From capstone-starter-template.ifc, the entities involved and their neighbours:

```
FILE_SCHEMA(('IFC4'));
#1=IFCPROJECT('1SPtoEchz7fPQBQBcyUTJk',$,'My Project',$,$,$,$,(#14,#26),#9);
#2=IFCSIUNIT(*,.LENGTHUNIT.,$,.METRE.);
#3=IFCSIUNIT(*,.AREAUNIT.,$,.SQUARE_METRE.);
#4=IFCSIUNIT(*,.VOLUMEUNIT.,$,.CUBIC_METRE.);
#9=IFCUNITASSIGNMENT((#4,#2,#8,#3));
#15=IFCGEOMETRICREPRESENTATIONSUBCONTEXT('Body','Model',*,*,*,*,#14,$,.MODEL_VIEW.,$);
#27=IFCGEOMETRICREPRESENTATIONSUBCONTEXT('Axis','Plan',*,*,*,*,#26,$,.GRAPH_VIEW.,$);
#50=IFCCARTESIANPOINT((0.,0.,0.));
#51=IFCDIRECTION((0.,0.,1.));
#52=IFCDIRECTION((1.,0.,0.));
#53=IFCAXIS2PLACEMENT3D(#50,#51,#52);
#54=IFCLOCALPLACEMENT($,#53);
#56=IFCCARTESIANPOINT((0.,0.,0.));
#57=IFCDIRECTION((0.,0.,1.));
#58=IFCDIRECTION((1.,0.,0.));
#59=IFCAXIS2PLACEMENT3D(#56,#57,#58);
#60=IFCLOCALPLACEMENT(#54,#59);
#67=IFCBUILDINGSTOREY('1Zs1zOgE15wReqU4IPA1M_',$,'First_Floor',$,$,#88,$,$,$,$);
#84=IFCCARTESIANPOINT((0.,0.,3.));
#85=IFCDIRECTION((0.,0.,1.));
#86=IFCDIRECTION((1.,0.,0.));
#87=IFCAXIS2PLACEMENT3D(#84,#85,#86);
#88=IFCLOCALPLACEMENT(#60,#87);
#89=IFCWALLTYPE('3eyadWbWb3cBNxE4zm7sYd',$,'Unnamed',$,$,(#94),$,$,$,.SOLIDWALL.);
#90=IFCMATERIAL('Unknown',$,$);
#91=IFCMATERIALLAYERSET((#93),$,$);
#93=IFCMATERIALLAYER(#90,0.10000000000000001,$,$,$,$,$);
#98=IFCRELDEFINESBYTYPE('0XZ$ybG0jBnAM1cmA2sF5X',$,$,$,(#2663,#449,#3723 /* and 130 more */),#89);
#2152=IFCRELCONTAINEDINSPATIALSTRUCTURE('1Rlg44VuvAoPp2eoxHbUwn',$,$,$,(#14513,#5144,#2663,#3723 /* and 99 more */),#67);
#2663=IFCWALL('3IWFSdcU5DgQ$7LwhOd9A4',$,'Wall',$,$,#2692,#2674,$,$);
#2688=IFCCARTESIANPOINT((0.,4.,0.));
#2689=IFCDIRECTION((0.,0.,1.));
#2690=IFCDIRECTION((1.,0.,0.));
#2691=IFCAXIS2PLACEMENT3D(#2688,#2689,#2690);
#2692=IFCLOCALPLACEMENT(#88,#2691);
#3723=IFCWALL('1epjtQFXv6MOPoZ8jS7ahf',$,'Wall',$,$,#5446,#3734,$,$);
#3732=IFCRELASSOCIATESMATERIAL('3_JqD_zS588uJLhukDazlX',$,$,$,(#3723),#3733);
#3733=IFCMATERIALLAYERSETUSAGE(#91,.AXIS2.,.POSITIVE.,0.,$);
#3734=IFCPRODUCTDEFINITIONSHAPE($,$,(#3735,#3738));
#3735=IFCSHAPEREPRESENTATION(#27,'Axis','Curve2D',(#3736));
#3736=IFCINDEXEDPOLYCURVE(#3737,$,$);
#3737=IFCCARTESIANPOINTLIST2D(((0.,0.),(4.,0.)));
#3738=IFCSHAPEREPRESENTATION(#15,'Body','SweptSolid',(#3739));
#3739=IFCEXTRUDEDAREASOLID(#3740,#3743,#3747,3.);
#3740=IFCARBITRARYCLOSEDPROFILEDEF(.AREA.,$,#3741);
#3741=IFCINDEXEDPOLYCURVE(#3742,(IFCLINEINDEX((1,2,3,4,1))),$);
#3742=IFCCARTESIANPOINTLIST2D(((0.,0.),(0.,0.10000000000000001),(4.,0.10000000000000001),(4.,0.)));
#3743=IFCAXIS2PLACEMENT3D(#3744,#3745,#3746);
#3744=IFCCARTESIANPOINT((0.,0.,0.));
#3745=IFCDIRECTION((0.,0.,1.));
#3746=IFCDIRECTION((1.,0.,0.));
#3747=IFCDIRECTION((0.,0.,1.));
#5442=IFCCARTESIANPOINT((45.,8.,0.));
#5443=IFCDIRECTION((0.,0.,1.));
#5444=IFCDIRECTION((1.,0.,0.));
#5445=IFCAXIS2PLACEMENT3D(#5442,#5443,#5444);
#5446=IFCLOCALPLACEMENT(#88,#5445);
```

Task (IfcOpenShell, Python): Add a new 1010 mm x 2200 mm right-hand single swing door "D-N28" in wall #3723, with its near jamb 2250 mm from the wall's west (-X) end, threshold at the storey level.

```python
import numpy as np
import ifcopenshell
import ifcopenshell.api.feature
import ifcopenshell.api.geometry
import ifcopenshell.api.root
import ifcopenshell.api.spatial
import ifcopenshell.geom
import ifcopenshell.util.element
import ifcopenshell.util.placement
import ifcopenshell.util.representation
import ifcopenshell.util.shape
import ifcopenshell.util.unit

model = ifcopenshell.open("capstone-starter-template.ifc")
unit_scale = ifcopenshell.util.unit.calculate_unit_scale(model)
settings = ifcopenshell.geom.settings()


def volume(element):
    """Net volume in cubic metres, openings subtracted."""
    shape = ifcopenshell.geom.create_shape(settings, element)
    return ifcopenshell.util.shape.get_volume(shape.geometry)


wall = model.by_guid("1epjtQFXv6MOPoZ8jS7ahf")
storey = ifcopenshell.util.element.get_container(wall, ifc_class="IfcBuildingStorey")
context = ifcopenshell.util.representation.get_context(model, "Model", "Body", "MODEL_VIEW")
before = volume(wall)

width, height, from_end, sill = 1.01, 2.2, 2.25, 0.0  # metres

# The wall runs along its own X axis, and the end named is its -X end.
wall_shape = ifcopenshell.geom.create_shape(settings, wall)
x, y, z = ifcopenshell.util.shape.get_vertices(wall_shape.geometry).T
start = x.min() + from_end
face, thickness = float(y.min()), float(y.max() - y.min())
wall_matrix = ifcopenshell.util.placement.get_local_placement(wall.ObjectPlacement)
level = ifcopenshell.util.placement.get_local_placement(storey.ObjectPlacement)[2, 3]


def in_wall(x, y):
    """Placement at x, y metres in the wall's axes, at sill height."""
    matrix = wall_matrix.copy()
    matrix[:, 3] = wall_matrix @ np.array([x / unit_scale, y / unit_scale, 0.0, 1.0])
    matrix[2, 3] = level + sill / unit_scale
    return matrix


# Opening: a box that overshoots both wall faces by 50 mm.
opening = ifcopenshell.api.root.create_entity(model, ifc_class="IfcOpeningElement", predefined_type="OPENING")
box = ifcopenshell.api.geometry.add_wall_representation(
    model, context=context, length=width, height=height, thickness=thickness + 0.1
)
ifcopenshell.api.geometry.assign_representation(model, product=opening, representation=box)
ifcopenshell.api.geometry.edit_object_placement(model, product=opening, matrix=in_wall(start, face - 0.05), is_si=False)
ifcopenshell.api.feature.add_feature(model, feature=opening, element=wall)

door = ifcopenshell.api.root.create_entity(model, ifc_class="IfcDoor", name="D-N28", predefined_type="DOOR")
door.OverallWidth, door.OverallHeight = width / unit_scale, height / unit_scale
door.OperationType = "SINGLE_SWING_RIGHT"
body = ifcopenshell.api.geometry.add_door_representation(
    model,
    context=context,
    overall_width=door.OverallWidth,
    overall_height=door.OverallHeight,
    operation_type="SINGLE_SWING_RIGHT",
    lining_properties={"LiningDepth": thickness / unit_scale, "ThresholdDepth": thickness / unit_scale},
)
ifcopenshell.api.geometry.assign_representation(model, product=door, representation=body)
ifcopenshell.api.spatial.assign_container(model, products=[door], relating_structure=storey)
ifcopenshell.api.feature.add_filling(model, opening=opening, element=door)

# The lining spans the wall, so the door starts at the wall face.
ifcopenshell.api.geometry.edit_object_placement(model, product=door, matrix=in_wall(start, face), is_si=False)

after = volume(wall)

print(f"wall volume {before:.3f} -> {after:.3f} m3")

model.write("capstone-starter-template_rev.ifc")
```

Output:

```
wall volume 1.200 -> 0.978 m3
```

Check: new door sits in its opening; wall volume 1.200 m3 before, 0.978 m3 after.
